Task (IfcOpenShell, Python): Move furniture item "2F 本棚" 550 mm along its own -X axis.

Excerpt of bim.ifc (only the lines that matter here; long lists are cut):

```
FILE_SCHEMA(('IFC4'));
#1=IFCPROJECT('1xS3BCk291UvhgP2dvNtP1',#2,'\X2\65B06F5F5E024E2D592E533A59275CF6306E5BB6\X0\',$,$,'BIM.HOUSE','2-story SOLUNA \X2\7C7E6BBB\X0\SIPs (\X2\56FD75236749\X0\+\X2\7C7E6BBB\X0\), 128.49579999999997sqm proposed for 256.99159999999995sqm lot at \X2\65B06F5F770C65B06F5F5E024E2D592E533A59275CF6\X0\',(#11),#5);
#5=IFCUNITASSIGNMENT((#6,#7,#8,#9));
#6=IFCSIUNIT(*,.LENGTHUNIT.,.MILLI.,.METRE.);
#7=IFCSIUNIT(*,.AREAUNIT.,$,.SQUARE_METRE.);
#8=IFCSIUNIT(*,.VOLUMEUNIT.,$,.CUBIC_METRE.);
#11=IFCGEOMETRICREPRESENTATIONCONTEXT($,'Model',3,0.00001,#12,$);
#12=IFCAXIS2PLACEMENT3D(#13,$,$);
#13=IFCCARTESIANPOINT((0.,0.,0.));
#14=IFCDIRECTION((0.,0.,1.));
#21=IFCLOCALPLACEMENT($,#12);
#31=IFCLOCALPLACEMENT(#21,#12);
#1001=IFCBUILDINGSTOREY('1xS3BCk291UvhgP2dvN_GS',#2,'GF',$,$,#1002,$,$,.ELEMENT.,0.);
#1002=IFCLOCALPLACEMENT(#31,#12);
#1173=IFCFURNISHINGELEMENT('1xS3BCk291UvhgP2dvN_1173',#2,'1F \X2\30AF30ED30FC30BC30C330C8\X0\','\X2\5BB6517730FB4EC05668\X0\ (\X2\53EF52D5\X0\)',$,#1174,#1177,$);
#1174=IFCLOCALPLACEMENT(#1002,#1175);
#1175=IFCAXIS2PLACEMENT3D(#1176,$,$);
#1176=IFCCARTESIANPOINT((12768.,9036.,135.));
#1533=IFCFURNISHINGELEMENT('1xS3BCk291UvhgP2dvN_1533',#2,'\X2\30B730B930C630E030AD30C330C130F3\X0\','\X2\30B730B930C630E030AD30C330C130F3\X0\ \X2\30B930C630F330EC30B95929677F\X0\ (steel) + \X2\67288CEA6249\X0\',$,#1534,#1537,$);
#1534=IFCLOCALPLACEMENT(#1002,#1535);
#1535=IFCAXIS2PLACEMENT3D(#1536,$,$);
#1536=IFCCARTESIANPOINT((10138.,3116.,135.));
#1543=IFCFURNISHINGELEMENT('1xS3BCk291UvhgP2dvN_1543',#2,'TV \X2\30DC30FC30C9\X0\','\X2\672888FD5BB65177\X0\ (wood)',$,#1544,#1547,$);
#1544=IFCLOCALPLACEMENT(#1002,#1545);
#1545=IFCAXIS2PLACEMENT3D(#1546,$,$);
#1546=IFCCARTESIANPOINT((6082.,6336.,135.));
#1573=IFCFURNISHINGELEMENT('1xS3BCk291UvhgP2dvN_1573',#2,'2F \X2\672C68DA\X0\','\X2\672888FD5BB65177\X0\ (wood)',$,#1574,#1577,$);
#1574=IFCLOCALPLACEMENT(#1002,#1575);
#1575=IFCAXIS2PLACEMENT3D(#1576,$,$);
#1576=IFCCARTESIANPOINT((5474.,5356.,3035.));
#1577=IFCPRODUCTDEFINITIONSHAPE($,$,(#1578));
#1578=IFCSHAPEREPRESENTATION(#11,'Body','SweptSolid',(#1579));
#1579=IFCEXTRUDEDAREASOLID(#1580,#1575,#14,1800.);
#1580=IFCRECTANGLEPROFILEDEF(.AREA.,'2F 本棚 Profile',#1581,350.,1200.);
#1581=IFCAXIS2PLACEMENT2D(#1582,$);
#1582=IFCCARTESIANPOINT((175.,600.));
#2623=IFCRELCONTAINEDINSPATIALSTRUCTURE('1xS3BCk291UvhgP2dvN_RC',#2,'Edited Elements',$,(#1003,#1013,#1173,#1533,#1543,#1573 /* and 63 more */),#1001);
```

```python
import ifcopenshell
import ifcopenshell.api.geometry
import ifcopenshell.util.placement

model = ifcopenshell.open("bim.ifc")

item = model.by_id(1573)
matrix = ifcopenshell.util.placement.get_local_placement(item.ObjectPlacement)
matrix[:3, 3] -= matrix[:3, 0] * 550.0
ifcopenshell.api.geometry.edit_object_placement(model, product=item, matrix=matrix, is_si=False)

print(ifcopenshell.util.placement.get_local_placement(item.ObjectPlacement).round(3) + 0.0)

model.write("bim-out.ifc")
```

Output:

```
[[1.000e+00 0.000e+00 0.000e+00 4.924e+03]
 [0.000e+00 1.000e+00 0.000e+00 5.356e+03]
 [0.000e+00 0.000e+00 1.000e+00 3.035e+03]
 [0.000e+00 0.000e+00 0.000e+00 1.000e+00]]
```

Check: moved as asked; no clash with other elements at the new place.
